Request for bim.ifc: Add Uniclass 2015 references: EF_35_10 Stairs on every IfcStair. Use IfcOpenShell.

First a look at what the model holds.

```python
import ifcopenshell

model = ifcopenshell.open("bim.ifc")
print(model.schema)
print("classifications:", [c.Name for c in model.by_type("IfcClassification")])
for ifc_class in ("IfcDoor", "IfcRoof", "IfcStair", "IfcWall", "IfcWindow"):
    print(ifc_class, len(model.by_type(ifc_class)))
```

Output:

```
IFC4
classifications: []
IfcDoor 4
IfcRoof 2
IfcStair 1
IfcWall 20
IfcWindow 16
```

```python
import ifcopenshell
import ifcopenshell.api.classification

model = ifcopenshell.open("bim.ifc")

system = ifcopenshell.api.classification.add_classification(model, classification="Uniclass 2015")

codes = {
    "IfcStair": ("EF_35_10", "Stairs"),
}
for ifc_class, (code, name) in codes.items():
    products = model.by_type(ifc_class)
    ifcopenshell.api.classification.add_reference(
        model, products=products, classification=system, identification=code, name=name
    )
    print(code, len(products))

model.write("bim_rev.ifc")
```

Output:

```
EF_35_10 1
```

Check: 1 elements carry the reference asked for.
